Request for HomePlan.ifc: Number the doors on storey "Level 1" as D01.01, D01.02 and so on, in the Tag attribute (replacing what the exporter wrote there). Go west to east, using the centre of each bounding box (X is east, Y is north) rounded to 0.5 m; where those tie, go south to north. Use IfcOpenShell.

First a look at what the model holds.

```python
import ifcopenshell
import ifcopenshell.util.element
import ifcopenshell.util.placement

model = ifcopenshell.open("HomePlan.ifc")
print(model.schema)
storey = next(s for s in model.by_type("IfcBuildingStorey") if s.Name == "Level 1")
doors = [e for e in ifcopenshell.util.element.get_decomposition(storey) if e.is_a("IfcDoor")]
for e in sorted(doors, key=lambda e: e.id()):
    origin = ifcopenshell.util.placement.get_local_placement(e.ObjectPlacement)[:3, 3]
    print(e.id(), e.Tag, e.Name, origin.round(2) + 0.0, sep=" | ")
```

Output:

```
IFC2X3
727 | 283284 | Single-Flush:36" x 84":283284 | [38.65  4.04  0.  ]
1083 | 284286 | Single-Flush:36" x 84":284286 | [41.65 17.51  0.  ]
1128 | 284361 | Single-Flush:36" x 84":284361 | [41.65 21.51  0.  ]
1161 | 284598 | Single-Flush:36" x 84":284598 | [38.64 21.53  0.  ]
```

```python
import ifcopenshell
import ifcopenshell.geom
import ifcopenshell.util.element
import ifcopenshell.util.shape

model = ifcopenshell.open("HomePlan.ifc")
settings = ifcopenshell.geom.settings()
settings.set("use-world-coords", True)


def centre(element):
    shape = ifcopenshell.geom.create_shape(settings, element)
    return ifcopenshell.util.shape.get_bbox_centroid(shape.geometry)


storey = next(s for s in model.by_type("IfcBuildingStorey") if s.Name == "Level 1")
doors = [e for e in ifcopenshell.util.element.get_decomposition(storey) if e.is_a("IfcDoor")]

# Insertion points can sit at a corner or the storey origin, so sort by the geometry (in metres).
centres = {e: centre(e) for e in doors}
doors.sort(key=lambda e: (round(centres[e][0] / 0.5), centres[e][1]))

for i, e in enumerate(doors, start=1):
    number = f"D01.{i:02d}"
    e.Tag = number
    print(e.id(), number)

model.write("HomePlan_v2.ifc")
```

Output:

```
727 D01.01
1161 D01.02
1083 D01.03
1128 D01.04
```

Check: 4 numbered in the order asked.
